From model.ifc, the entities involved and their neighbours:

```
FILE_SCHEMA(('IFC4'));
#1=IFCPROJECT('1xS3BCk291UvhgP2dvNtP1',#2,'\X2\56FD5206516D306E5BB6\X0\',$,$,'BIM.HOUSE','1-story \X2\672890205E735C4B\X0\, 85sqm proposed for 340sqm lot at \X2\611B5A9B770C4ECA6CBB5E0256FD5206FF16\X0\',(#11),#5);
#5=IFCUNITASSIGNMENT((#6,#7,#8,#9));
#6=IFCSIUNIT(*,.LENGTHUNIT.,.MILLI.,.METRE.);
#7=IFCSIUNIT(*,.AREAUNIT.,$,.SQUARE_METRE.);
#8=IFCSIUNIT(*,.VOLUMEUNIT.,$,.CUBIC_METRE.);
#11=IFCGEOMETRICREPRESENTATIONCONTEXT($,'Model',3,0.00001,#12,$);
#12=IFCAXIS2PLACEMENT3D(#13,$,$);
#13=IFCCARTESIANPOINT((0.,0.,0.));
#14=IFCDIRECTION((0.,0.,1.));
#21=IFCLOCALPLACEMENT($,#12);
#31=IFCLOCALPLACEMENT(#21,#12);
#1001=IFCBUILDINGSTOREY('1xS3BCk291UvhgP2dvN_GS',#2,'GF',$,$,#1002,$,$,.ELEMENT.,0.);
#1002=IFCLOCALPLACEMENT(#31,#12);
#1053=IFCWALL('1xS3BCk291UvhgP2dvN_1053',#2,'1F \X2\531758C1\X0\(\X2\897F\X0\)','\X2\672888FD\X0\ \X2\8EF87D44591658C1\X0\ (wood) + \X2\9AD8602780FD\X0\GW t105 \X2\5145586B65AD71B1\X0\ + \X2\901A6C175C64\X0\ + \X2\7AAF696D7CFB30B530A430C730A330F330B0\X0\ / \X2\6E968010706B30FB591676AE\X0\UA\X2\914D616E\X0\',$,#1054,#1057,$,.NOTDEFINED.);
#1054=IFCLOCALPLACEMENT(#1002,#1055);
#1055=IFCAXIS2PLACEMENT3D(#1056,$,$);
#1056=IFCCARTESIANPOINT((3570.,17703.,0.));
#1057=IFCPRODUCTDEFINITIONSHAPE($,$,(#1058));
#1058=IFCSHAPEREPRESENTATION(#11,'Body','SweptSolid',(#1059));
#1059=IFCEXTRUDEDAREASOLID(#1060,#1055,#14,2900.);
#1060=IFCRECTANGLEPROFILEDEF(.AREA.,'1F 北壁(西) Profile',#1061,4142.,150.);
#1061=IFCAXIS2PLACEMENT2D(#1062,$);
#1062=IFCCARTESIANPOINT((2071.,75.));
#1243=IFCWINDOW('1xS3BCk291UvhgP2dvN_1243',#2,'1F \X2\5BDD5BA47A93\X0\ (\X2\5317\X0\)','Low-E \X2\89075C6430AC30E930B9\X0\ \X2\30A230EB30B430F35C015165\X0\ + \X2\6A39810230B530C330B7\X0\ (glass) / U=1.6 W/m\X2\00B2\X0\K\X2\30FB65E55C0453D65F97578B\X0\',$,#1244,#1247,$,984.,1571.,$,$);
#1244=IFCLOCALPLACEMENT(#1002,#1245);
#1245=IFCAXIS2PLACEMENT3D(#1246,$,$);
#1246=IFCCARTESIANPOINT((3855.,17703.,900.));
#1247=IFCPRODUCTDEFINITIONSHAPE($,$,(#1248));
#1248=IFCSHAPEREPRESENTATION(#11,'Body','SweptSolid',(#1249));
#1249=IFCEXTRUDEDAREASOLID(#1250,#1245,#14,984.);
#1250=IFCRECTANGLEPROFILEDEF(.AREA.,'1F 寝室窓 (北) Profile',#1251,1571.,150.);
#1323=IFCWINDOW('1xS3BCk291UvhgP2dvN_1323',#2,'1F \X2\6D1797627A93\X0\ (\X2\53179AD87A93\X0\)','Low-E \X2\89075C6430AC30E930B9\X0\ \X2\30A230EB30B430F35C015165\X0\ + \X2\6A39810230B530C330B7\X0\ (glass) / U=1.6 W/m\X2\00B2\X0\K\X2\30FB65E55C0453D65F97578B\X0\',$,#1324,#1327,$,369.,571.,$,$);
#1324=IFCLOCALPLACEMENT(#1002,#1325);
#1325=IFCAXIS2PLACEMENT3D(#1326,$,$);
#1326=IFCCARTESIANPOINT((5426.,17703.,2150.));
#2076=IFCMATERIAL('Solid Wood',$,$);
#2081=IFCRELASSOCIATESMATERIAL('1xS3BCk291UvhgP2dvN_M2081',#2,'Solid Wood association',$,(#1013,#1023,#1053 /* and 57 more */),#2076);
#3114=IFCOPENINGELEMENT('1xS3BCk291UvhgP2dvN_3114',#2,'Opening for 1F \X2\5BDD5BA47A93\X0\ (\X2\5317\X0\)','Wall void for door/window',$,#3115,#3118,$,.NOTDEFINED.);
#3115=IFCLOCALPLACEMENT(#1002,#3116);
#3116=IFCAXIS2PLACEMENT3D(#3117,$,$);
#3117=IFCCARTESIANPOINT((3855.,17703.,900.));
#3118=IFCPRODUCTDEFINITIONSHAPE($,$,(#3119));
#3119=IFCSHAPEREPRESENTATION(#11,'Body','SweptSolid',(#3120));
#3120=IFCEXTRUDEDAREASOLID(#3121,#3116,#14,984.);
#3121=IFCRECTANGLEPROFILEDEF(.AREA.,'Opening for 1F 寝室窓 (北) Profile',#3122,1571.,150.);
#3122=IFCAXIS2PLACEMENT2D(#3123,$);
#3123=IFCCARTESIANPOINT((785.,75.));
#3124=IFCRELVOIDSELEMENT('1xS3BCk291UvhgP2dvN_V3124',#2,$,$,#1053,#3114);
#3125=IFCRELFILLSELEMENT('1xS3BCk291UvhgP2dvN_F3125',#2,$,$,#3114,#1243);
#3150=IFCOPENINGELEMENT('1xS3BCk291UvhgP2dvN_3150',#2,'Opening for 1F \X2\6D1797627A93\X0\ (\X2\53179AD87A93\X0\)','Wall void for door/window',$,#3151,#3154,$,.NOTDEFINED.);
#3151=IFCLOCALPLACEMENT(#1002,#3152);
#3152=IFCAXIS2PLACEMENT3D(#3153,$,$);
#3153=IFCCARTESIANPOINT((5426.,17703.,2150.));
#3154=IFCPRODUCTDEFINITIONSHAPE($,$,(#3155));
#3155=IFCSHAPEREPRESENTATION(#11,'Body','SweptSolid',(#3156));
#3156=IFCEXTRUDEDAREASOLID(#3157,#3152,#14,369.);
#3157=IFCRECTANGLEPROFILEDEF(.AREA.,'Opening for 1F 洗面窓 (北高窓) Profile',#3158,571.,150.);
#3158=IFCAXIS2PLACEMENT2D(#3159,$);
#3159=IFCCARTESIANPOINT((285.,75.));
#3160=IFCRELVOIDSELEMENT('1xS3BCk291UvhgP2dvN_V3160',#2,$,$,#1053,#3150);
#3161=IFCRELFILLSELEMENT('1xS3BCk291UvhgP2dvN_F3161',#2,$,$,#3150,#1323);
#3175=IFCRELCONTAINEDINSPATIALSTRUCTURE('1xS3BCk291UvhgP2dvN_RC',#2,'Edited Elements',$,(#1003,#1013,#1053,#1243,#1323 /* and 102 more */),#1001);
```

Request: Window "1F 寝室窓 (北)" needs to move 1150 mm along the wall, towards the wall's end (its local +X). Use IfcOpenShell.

```python
import ifcopenshell
import ifcopenshell.api.geometry
import ifcopenshell.util.placement
import ifcopenshell.util.unit

model = ifcopenshell.open("model.ifc")
unit_scale = ifcopenshell.util.unit.calculate_unit_scale(model)

window = model.by_id(1243)
opening = window.FillsVoids[0].RelatingOpeningElement
wall = opening.VoidsElements[0].RelatingBuildingElement

wall_matrix = ifcopenshell.util.placement.get_local_placement(wall.ObjectPlacement)
shift = wall_matrix[:3, 0] * 1.15 / unit_scale
before = ifcopenshell.util.placement.get_local_placement(window.ObjectPlacement)[:3, 3].copy()

# The window is not placed relative to its opening, so move both.
for product in (opening, window):
    matrix = ifcopenshell.util.placement.get_local_placement(product.ObjectPlacement)
    matrix[:3, 3] += shift
    ifcopenshell.api.geometry.edit_object_placement(model, product=product, matrix=matrix, is_si=False)

after = ifcopenshell.util.placement.get_local_placement(window.ObjectPlacement)[:3, 3]
print("window moved by", (after - before).round(3) + 0.0)

model.write("model_v2.ifc")
```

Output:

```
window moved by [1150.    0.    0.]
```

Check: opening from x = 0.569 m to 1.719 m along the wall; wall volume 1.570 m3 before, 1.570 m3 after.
